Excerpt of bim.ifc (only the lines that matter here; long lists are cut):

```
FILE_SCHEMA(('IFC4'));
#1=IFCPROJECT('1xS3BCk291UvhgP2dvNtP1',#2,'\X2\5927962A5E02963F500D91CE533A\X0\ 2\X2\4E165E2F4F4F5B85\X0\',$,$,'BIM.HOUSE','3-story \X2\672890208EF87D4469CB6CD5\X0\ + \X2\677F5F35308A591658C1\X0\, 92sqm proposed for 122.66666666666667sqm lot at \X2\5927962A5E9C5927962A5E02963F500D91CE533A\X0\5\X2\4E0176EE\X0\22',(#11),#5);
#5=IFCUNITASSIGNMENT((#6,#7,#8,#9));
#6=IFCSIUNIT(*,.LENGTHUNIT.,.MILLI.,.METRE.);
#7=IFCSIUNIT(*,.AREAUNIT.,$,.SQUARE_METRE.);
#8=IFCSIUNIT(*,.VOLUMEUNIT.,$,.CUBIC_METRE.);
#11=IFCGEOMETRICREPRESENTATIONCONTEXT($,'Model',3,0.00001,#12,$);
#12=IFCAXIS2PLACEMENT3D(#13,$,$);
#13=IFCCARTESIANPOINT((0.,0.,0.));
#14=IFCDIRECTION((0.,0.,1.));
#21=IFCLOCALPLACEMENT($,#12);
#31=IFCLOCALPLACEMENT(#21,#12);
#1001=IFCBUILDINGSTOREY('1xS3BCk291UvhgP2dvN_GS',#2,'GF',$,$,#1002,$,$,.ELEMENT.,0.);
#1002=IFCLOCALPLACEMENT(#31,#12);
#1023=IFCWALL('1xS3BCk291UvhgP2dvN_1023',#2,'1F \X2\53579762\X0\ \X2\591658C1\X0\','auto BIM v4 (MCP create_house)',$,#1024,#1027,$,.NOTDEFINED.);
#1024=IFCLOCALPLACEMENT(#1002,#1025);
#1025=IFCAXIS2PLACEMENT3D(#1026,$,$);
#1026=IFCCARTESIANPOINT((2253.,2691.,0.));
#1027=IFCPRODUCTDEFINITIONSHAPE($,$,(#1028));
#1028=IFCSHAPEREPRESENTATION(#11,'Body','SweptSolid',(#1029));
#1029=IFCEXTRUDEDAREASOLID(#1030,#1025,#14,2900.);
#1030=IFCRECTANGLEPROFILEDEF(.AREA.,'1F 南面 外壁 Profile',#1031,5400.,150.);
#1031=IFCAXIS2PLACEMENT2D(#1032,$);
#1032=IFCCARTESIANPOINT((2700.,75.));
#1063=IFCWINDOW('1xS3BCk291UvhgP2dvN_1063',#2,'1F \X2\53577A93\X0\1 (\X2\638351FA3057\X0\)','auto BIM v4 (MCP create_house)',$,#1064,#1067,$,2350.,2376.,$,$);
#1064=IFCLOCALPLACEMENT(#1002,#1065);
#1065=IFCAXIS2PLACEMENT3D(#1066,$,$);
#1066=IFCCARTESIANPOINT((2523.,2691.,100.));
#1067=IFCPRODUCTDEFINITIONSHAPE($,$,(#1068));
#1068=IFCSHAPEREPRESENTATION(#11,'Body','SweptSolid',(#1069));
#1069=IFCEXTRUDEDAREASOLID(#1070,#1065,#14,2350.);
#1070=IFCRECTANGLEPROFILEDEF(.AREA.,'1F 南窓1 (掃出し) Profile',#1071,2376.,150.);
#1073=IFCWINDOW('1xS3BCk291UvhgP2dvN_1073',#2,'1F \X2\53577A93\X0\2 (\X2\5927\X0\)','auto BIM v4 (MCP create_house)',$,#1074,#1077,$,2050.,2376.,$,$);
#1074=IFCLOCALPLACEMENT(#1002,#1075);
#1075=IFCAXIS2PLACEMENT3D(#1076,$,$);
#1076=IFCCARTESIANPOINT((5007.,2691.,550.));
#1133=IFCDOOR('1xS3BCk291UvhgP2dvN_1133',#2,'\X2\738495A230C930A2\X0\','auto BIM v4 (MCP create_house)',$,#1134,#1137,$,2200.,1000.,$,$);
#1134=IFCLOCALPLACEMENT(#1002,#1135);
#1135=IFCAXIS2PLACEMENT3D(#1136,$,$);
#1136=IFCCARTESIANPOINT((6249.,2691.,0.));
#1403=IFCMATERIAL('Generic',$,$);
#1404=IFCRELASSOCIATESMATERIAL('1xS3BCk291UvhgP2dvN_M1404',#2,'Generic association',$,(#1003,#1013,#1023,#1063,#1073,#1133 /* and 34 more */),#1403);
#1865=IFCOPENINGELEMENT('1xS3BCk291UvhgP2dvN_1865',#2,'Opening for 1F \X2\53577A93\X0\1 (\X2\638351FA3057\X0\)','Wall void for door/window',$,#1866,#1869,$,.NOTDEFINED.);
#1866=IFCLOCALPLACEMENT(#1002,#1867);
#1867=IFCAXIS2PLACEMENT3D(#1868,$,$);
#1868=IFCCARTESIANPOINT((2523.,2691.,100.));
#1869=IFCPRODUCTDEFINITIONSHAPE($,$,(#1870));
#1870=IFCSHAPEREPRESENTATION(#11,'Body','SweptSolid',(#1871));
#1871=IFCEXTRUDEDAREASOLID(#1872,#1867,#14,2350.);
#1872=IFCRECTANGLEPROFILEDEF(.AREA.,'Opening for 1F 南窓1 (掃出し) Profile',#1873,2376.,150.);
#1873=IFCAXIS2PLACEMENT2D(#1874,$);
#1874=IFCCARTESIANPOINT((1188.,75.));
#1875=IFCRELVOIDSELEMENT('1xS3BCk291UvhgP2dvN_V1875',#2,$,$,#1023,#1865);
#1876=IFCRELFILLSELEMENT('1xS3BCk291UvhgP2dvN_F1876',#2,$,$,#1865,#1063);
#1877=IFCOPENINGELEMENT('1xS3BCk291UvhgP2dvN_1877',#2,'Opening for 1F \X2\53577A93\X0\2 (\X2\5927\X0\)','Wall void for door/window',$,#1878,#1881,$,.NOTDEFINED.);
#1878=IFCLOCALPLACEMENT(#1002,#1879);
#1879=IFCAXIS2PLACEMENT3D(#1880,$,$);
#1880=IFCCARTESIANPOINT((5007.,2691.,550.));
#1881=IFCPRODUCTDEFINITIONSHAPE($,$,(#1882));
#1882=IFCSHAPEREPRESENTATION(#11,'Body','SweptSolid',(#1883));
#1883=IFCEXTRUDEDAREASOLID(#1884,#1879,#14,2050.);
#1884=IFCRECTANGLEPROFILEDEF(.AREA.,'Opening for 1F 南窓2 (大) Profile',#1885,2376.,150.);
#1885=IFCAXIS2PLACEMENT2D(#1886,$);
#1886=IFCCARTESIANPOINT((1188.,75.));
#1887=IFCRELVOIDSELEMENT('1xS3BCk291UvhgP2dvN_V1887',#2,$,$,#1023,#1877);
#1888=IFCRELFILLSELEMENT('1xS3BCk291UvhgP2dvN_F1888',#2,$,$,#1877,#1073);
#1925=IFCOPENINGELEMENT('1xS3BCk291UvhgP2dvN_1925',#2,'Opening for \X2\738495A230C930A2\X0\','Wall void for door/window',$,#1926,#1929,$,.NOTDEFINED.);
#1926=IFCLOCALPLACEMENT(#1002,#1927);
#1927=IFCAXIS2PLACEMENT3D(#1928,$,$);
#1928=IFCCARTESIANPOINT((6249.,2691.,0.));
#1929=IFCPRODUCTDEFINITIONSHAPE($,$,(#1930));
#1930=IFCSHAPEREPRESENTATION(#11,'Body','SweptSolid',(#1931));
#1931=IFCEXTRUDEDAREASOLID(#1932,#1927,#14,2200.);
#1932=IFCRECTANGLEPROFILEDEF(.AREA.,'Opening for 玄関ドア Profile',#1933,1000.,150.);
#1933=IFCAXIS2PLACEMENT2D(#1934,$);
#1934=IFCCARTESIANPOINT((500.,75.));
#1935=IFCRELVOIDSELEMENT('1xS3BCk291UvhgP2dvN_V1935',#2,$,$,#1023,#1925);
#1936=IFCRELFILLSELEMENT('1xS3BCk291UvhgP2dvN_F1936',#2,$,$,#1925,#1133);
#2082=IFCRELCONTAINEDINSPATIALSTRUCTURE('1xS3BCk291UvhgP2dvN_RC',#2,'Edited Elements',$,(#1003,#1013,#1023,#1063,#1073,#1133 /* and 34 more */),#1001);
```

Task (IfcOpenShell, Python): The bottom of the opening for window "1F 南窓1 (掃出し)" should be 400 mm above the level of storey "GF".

```python
import numpy as np
import ifcopenshell
import ifcopenshell.api.geometry
import ifcopenshell.geom
import ifcopenshell.util.element
import ifcopenshell.util.placement
import ifcopenshell.util.shape
import ifcopenshell.util.unit

model = ifcopenshell.open("bim.ifc")
unit_scale = ifcopenshell.util.unit.calculate_unit_scale(model)

window = model.by_guid("1xS3BCk291UvhgP2dvN_1063")
opening = window.FillsVoids[0].RelatingOpeningElement
storey = ifcopenshell.util.element.get_container(window, ifc_class="IfcBuildingStorey")
level = ifcopenshell.util.placement.get_local_placement(storey.ObjectPlacement)[2, 3]

# The opening's origin need not be at the sill, so measure its lowest point.
shape = ifcopenshell.geom.create_shape(ifcopenshell.geom.settings(), opening)
bottom = ifcopenshell.util.shape.get_shape_bottom_elevation(shape, shape.geometry) / unit_scale
dz = level + 400.0 - bottom

shift = np.array([0.0, 0.0, dz])
# The window is not placed relative to its opening, so move both.
for product in (opening, window):
    matrix = ifcopenshell.util.placement.get_local_placement(product.ObjectPlacement)
    matrix[:3, 3] += shift
    ifcopenshell.api.geometry.edit_object_placement(model, product=product, matrix=matrix, is_si=False)

print(f"moved by {dz * unit_scale:+.3f} m")

model.write("bim-out.ifc")
```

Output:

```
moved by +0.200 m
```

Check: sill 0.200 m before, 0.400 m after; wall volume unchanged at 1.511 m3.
